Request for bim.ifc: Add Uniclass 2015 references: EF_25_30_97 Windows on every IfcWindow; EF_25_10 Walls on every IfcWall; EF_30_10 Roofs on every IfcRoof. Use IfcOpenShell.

First a look at what the model holds.

```python
import ifcopenshell

model = ifcopenshell.open("bim.ifc")
print(model.schema)
print("classifications:", [c.Name for c in model.by_type("IfcClassification")])
for ifc_class in ("IfcDoor", "IfcRoof", "IfcStair", "IfcWall", "IfcWindow"):
    print(ifc_class, len(model.by_type(ifc_class)))
```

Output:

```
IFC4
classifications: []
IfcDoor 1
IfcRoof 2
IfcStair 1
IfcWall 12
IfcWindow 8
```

```python
import ifcopenshell
import ifcopenshell.api.classification

model = ifcopenshell.open("bim.ifc")

system = ifcopenshell.api.classification.add_classification(model, classification="Uniclass 2015")

codes = {
    "IfcWindow": ("EF_25_30_97", "Windows"),
    "IfcWall": ("EF_25_10", "Walls"),
    "IfcRoof": ("EF_30_10", "Roofs"),
}
for ifc_class, (code, name) in codes.items():
    products = model.by_type(ifc_class)
    ifcopenshell.api.classification.add_reference(
        model, products=products, classification=system, identification=code, name=name
    )
    print(code, len(products))

model.write("bim-out.ifc")
```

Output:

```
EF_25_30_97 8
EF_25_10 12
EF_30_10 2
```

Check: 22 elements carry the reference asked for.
